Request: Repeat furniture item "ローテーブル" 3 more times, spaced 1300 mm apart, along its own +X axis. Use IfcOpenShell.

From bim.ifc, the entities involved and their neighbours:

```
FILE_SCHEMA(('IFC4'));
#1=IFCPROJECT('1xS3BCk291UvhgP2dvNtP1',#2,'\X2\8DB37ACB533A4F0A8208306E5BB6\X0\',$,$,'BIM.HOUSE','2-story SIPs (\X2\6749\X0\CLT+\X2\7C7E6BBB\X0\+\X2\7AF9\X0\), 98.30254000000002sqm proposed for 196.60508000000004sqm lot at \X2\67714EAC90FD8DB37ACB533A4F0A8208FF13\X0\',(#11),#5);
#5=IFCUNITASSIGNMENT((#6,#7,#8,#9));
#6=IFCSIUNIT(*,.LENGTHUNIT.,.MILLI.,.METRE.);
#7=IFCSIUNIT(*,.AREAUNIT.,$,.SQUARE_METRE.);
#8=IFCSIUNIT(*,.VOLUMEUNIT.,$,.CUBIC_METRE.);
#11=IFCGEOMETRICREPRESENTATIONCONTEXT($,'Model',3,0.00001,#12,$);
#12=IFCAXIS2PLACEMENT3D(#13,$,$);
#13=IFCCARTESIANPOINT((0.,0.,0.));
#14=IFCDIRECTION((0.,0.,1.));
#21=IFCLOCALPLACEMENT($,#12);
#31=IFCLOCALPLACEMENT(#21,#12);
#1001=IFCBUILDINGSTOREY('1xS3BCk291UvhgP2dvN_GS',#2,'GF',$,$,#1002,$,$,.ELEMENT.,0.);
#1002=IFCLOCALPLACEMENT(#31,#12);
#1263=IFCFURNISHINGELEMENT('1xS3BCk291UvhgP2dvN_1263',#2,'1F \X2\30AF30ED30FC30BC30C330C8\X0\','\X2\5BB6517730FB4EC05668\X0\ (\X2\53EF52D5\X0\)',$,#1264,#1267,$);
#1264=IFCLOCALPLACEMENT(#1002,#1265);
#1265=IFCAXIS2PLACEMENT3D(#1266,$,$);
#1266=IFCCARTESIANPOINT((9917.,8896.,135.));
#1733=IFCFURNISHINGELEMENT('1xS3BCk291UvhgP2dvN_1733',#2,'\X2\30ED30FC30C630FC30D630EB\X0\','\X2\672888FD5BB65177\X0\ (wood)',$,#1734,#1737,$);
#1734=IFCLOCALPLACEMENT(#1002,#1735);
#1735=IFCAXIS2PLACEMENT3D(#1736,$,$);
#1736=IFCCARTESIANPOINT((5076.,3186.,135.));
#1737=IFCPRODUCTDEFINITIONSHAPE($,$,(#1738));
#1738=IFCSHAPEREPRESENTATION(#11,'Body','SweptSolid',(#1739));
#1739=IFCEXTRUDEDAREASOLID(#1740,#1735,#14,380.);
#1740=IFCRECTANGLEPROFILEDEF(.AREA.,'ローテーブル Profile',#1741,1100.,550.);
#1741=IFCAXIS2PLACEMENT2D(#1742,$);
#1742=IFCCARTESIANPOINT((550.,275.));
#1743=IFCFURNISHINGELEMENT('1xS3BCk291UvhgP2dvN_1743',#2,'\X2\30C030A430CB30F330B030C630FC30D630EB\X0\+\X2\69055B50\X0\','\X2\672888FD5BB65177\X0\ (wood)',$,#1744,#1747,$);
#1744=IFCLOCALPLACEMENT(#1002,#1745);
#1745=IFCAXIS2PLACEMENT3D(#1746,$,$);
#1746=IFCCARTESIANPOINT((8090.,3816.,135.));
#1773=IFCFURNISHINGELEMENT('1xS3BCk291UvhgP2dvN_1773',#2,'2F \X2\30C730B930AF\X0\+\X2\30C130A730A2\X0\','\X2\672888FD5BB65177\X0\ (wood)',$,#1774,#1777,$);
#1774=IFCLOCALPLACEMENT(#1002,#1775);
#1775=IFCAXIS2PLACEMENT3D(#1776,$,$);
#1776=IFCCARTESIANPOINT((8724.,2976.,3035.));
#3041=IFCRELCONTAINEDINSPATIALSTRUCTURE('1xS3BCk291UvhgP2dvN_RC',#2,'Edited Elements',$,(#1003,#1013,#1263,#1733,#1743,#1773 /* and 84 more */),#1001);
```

```python
import ifcopenshell
import ifcopenshell.api.geometry
import ifcopenshell.api.root
import ifcopenshell.util.element
import ifcopenshell.util.placement
import ifcopenshell.util.unit

model = ifcopenshell.open("bim.ifc")
unit_scale = ifcopenshell.util.unit.calculate_unit_scale(model)


def reuse_history(source, copy):
    """copy_class also copies each property set's owner history, people and application; keep the originals."""
    for rel in copy.IsDefinedBy:
        if rel.is_a("IfcRelDefinesByProperties") and (history := rel.RelatingPropertyDefinition.OwnerHistory):
            rel.RelatingPropertyDefinition.OwnerHistory = source.OwnerHistory
            ifcopenshell.util.element.remove_deep2(model, history)


source = model.by_id(1733)
base = ifcopenshell.util.placement.get_local_placement(source.ObjectPlacement)
step = base[:3, 0] * 1.3 / unit_scale

for i in range(1, 4):
    copy = ifcopenshell.api.root.copy_class(model, product=source)
    copy.Representation = ifcopenshell.util.element.copy_deep(
        model, source.Representation, exclude=["IfcGeometricRepresentationContext", "IfcRepresentationMap"]
    )
    reuse_history(source, copy)
    matrix = base.copy()
    matrix[:3, 3] += i * step
    print("added at", matrix[:3, 3].round(3) + 0.0)
    ifcopenshell.api.geometry.edit_object_placement(model, product=copy, matrix=matrix, is_si=False)

model.write("bim_v2.ifc")
```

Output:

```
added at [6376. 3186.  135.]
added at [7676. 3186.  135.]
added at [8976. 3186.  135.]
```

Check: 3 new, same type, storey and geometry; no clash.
